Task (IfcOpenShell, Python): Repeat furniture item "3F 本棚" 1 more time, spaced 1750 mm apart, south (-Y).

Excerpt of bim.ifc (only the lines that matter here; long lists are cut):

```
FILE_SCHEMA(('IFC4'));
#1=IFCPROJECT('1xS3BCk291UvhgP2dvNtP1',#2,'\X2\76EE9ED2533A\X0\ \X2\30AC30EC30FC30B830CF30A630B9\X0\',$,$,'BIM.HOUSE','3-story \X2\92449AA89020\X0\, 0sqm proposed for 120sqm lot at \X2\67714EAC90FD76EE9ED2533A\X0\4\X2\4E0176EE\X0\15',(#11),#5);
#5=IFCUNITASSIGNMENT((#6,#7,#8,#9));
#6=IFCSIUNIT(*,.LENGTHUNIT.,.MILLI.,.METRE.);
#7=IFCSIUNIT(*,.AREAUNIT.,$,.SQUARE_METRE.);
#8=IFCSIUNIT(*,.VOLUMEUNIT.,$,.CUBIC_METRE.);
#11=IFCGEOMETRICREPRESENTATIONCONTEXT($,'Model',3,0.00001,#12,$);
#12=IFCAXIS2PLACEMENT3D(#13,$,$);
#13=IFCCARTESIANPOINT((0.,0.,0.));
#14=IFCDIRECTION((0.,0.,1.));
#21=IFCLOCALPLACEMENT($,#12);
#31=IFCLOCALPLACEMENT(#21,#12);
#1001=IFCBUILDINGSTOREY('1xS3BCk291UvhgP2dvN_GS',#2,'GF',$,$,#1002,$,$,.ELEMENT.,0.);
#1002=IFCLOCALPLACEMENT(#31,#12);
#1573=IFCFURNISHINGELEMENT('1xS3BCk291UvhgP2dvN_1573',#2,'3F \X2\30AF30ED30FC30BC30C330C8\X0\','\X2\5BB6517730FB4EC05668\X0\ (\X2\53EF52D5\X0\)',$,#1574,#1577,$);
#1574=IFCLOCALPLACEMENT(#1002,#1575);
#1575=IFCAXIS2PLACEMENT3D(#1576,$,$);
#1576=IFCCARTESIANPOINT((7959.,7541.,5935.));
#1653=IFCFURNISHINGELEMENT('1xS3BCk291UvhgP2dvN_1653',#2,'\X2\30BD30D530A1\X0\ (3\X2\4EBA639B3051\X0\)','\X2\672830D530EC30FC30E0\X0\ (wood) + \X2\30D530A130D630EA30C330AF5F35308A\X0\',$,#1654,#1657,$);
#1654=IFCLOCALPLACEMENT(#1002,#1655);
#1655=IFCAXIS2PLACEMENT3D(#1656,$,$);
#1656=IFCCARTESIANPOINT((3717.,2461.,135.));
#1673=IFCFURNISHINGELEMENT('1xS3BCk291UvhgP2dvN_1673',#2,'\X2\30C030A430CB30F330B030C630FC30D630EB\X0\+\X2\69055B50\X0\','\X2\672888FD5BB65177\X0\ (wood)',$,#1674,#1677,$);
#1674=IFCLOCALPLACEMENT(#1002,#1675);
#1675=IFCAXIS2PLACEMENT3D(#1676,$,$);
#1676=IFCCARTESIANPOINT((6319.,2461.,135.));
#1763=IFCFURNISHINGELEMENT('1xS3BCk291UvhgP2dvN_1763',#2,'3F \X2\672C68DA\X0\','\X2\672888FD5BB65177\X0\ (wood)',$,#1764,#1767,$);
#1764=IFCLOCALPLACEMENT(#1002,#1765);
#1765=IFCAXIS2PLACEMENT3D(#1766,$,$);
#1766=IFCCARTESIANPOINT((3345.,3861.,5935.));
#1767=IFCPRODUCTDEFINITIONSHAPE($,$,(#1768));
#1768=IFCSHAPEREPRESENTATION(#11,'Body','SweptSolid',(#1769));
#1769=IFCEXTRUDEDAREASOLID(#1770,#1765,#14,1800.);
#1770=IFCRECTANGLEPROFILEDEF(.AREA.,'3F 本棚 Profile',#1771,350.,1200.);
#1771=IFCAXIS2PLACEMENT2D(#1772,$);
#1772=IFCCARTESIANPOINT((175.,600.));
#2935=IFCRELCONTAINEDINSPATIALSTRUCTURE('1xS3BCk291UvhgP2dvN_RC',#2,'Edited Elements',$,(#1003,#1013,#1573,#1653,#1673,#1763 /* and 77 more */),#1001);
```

```python
import numpy as np
import ifcopenshell
import ifcopenshell.api.geometry
import ifcopenshell.api.root
import ifcopenshell.util.element
import ifcopenshell.util.placement

model = ifcopenshell.open("bim.ifc")


def reuse_history(source, copy):
    """copy_class also copies each property set's owner history, people and application; keep the originals."""
    for rel in copy.IsDefinedBy:
        if rel.is_a("IfcRelDefinesByProperties") and (history := rel.RelatingPropertyDefinition.OwnerHistory):
            rel.RelatingPropertyDefinition.OwnerHistory = source.OwnerHistory
            ifcopenshell.util.element.remove_deep2(model, history)


source = model.by_guid("1xS3BCk291UvhgP2dvN_1763")
base = ifcopenshell.util.placement.get_local_placement(source.ObjectPlacement)
step = np.array([0.0, -1.0, 0.0]) * 1750.0

for i in range(1, 2):
    copy = ifcopenshell.api.root.copy_class(model, product=source)
    copy.Representation = ifcopenshell.util.element.copy_deep(
        model, source.Representation, exclude=["IfcGeometricRepresentationContext", "IfcRepresentationMap"]
    )
    reuse_history(source, copy)
    matrix = base.copy()
    matrix[:3, 3] += i * step
    print("added at", matrix[:3, 3].round(3) + 0.0)
    ifcopenshell.api.geometry.edit_object_placement(model, product=copy, matrix=matrix, is_si=False)

model.write("bim_updated.ifc")
```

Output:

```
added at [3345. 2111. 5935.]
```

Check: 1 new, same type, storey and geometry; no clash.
